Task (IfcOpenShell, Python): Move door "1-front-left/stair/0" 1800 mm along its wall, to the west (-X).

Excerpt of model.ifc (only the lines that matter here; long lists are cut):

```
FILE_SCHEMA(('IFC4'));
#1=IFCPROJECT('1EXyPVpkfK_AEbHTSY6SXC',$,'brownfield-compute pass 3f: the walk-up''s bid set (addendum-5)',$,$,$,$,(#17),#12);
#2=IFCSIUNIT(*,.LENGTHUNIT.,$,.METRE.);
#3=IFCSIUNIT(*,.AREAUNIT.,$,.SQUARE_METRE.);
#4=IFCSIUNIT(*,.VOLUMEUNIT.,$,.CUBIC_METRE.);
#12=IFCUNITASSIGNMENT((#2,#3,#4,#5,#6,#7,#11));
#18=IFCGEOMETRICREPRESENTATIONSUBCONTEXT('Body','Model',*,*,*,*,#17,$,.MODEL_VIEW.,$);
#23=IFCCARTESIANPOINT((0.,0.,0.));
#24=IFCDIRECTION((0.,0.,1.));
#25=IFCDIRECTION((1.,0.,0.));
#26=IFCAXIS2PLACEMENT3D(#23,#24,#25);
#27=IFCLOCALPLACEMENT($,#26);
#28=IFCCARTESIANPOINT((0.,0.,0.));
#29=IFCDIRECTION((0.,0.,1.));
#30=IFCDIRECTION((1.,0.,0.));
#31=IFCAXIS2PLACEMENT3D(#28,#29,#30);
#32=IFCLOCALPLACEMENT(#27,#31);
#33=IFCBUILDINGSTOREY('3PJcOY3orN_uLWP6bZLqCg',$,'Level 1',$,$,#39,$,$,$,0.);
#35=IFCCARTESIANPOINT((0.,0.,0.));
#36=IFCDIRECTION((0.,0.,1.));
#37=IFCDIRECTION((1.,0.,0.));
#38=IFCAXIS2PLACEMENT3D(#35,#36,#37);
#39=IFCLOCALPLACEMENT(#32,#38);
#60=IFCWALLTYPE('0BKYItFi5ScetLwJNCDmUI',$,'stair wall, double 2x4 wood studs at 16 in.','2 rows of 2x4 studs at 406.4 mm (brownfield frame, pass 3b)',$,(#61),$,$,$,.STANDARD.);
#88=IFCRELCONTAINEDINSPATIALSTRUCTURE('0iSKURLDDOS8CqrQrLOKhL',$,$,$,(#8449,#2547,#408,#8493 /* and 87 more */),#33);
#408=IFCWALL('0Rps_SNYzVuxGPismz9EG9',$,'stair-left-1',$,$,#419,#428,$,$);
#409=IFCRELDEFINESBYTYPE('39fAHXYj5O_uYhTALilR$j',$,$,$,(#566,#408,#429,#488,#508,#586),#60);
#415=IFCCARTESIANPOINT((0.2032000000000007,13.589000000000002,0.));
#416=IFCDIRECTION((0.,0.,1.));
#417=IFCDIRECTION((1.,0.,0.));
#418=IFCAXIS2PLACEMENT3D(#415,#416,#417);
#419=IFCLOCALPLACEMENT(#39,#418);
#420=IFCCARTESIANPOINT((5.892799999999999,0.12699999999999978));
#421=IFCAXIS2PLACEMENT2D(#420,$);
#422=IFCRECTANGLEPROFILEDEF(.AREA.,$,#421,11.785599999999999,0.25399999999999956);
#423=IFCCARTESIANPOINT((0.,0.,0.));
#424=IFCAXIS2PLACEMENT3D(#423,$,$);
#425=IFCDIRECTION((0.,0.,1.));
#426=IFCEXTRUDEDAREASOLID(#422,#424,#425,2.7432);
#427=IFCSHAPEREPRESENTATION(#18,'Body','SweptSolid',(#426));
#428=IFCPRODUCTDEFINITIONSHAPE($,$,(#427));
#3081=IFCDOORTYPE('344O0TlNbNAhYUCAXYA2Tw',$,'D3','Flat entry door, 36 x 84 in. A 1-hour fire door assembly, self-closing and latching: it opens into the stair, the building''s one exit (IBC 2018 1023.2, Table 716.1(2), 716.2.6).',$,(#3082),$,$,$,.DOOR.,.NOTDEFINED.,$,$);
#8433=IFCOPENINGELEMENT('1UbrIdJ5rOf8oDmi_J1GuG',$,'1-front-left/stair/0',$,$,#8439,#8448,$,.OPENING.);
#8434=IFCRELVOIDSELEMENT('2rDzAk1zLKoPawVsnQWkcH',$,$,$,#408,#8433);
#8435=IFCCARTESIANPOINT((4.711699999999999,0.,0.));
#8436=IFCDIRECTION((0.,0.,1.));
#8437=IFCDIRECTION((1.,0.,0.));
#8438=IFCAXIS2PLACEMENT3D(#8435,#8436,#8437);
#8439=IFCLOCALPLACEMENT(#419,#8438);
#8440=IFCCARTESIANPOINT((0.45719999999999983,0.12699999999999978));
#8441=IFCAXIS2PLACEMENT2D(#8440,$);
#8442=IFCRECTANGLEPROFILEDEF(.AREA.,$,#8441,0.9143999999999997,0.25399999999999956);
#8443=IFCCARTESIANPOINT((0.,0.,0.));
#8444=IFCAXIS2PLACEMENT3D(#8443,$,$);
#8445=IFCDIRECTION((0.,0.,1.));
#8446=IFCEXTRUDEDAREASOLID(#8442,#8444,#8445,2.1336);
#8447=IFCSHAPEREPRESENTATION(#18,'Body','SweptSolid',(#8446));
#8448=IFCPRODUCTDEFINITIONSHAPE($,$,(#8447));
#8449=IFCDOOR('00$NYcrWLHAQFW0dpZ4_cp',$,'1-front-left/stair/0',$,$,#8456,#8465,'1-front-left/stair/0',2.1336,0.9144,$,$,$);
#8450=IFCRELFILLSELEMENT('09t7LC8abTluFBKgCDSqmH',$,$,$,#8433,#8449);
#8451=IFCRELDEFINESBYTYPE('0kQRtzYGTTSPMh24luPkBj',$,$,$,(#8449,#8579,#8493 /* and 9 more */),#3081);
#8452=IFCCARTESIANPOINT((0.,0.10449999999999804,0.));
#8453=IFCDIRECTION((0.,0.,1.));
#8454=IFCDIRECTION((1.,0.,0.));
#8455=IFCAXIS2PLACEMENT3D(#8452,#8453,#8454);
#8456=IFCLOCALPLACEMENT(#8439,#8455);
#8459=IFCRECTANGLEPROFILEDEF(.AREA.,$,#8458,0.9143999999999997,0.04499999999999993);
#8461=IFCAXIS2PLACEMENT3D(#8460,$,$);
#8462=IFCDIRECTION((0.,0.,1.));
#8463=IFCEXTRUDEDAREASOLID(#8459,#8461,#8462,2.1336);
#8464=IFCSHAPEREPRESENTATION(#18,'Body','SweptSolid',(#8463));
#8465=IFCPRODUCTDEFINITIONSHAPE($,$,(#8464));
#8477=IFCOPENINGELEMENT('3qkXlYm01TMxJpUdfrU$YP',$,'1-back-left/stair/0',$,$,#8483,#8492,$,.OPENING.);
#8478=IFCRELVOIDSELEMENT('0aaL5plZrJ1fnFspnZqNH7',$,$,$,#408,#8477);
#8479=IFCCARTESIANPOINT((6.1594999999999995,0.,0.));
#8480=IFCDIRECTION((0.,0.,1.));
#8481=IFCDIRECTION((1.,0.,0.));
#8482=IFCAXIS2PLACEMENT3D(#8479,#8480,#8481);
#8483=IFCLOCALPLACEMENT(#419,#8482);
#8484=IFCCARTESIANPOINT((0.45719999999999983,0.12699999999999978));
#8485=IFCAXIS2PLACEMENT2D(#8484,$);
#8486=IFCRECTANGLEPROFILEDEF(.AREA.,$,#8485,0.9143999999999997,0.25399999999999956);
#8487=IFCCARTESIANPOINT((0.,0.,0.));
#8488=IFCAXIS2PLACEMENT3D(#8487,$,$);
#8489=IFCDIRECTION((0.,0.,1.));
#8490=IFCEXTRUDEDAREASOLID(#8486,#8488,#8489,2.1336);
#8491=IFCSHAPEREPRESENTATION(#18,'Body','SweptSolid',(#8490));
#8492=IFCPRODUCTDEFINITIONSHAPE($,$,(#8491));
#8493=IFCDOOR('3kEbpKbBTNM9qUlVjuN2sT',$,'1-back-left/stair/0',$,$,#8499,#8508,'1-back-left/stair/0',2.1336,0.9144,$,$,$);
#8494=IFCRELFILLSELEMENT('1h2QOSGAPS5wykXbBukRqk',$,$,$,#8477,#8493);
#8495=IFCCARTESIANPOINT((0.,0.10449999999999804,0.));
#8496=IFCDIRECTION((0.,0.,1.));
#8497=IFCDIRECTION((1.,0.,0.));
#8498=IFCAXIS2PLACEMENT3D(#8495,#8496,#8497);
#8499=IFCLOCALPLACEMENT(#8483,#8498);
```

```python
import ifcopenshell
import ifcopenshell.api.geometry
import ifcopenshell.util.placement

model = ifcopenshell.open("model.ifc")

door = model.by_id(8449)
opening = door.FillsVoids[0].RelatingOpeningElement
wall = opening.VoidsElements[0].RelatingBuildingElement

wall_matrix = ifcopenshell.util.placement.get_local_placement(wall.ObjectPlacement)
shift = wall_matrix[:3, 0] * -1.8
before = ifcopenshell.util.placement.get_local_placement(door.ObjectPlacement)[:3, 3].copy()

# The door is placed relative to its opening, so it follows when the opening moves.
matrix = ifcopenshell.util.placement.get_local_placement(opening.ObjectPlacement)
matrix[:3, 3] += shift
ifcopenshell.api.geometry.edit_object_placement(
    model, product=opening, matrix=matrix, is_si=False, should_transform_children=True
)

after = ifcopenshell.util.placement.get_local_placement(door.ObjectPlacement)[:3, 3]
print("door moved by", (after - before).round(3) + 0.0)

model.write("model_updated.ifc")
```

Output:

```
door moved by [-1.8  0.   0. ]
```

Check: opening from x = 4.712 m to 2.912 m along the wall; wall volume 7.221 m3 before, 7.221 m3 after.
